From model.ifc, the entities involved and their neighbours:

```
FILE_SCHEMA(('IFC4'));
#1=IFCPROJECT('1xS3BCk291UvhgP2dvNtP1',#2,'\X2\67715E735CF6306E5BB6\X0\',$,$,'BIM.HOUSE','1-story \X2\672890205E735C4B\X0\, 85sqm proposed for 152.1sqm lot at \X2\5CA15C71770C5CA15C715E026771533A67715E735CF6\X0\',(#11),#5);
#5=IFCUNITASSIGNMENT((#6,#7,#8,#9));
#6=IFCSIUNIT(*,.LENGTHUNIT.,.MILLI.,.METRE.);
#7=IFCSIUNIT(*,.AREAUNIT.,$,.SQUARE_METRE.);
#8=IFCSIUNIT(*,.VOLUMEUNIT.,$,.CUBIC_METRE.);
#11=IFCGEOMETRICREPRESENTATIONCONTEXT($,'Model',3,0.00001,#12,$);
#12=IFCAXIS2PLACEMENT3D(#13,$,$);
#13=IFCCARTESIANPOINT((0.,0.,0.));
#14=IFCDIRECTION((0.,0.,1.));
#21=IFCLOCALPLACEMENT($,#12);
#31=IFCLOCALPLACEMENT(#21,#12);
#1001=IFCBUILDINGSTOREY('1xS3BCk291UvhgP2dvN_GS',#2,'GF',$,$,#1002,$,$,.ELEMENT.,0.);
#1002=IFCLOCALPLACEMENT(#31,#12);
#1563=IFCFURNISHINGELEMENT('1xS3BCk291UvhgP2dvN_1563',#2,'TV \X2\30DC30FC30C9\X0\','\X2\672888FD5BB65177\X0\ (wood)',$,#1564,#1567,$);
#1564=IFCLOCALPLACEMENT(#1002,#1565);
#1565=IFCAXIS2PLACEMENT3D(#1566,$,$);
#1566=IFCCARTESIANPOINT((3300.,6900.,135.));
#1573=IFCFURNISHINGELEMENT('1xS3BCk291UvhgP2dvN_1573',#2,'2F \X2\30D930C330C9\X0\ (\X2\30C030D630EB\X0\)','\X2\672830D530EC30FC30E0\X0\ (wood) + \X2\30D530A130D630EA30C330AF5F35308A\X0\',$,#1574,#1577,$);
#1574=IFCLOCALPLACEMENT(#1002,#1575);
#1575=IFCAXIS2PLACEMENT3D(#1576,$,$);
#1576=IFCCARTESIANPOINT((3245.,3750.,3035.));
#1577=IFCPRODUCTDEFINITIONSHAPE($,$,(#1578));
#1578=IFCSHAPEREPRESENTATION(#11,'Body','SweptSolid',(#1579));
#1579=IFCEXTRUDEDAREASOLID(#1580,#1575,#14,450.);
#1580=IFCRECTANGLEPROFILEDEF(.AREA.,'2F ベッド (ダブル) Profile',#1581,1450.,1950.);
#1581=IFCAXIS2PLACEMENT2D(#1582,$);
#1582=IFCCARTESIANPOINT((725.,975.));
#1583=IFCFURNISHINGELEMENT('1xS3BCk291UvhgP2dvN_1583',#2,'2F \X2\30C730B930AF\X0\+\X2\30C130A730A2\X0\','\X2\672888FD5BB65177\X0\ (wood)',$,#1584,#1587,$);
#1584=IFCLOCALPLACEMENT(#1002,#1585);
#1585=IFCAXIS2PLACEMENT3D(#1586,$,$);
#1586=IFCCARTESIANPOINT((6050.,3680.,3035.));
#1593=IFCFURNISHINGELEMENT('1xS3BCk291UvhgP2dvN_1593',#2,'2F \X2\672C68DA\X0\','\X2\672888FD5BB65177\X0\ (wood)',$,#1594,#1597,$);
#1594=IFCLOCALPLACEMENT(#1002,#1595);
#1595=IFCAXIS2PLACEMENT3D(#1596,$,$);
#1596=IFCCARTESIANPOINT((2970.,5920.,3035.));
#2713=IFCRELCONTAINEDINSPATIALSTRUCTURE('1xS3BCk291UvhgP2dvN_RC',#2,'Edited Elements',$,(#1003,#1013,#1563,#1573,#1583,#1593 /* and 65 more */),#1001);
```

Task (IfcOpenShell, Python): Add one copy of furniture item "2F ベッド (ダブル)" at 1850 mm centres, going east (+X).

```python
import numpy as np
import ifcopenshell
import ifcopenshell.api.geometry
import ifcopenshell.api.root
import ifcopenshell.util.element
import ifcopenshell.util.placement

model = ifcopenshell.open("model.ifc")


def reuse_history(source, copy):
    """copy_class also copies each property set's owner history, people and application; keep the originals."""
    for rel in copy.IsDefinedBy:
        if rel.is_a("IfcRelDefinesByProperties") and (history := rel.RelatingPropertyDefinition.OwnerHistory):
            rel.RelatingPropertyDefinition.OwnerHistory = source.OwnerHistory
            ifcopenshell.util.element.remove_deep2(model, history)


source = model.by_id(1573)
base = ifcopenshell.util.placement.get_local_placement(source.ObjectPlacement)
step = np.array([1.0, 0.0, 0.0]) * 1850.0

for i in range(1, 2):
    copy = ifcopenshell.api.root.copy_class(model, product=source)
    copy.Representation = ifcopenshell.util.element.copy_deep(
        model, source.Representation, exclude=["IfcGeometricRepresentationContext", "IfcRepresentationMap"]
    )
    reuse_history(source, copy)
    matrix = base.copy()
    matrix[:3, 3] += i * step
    print("added at", matrix[:3, 3].round(3) + 0.0)
    ifcopenshell.api.geometry.edit_object_placement(model, product=copy, matrix=matrix, is_si=False)

model.write("model_edited.ifc")
```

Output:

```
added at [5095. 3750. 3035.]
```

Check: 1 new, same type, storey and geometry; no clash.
